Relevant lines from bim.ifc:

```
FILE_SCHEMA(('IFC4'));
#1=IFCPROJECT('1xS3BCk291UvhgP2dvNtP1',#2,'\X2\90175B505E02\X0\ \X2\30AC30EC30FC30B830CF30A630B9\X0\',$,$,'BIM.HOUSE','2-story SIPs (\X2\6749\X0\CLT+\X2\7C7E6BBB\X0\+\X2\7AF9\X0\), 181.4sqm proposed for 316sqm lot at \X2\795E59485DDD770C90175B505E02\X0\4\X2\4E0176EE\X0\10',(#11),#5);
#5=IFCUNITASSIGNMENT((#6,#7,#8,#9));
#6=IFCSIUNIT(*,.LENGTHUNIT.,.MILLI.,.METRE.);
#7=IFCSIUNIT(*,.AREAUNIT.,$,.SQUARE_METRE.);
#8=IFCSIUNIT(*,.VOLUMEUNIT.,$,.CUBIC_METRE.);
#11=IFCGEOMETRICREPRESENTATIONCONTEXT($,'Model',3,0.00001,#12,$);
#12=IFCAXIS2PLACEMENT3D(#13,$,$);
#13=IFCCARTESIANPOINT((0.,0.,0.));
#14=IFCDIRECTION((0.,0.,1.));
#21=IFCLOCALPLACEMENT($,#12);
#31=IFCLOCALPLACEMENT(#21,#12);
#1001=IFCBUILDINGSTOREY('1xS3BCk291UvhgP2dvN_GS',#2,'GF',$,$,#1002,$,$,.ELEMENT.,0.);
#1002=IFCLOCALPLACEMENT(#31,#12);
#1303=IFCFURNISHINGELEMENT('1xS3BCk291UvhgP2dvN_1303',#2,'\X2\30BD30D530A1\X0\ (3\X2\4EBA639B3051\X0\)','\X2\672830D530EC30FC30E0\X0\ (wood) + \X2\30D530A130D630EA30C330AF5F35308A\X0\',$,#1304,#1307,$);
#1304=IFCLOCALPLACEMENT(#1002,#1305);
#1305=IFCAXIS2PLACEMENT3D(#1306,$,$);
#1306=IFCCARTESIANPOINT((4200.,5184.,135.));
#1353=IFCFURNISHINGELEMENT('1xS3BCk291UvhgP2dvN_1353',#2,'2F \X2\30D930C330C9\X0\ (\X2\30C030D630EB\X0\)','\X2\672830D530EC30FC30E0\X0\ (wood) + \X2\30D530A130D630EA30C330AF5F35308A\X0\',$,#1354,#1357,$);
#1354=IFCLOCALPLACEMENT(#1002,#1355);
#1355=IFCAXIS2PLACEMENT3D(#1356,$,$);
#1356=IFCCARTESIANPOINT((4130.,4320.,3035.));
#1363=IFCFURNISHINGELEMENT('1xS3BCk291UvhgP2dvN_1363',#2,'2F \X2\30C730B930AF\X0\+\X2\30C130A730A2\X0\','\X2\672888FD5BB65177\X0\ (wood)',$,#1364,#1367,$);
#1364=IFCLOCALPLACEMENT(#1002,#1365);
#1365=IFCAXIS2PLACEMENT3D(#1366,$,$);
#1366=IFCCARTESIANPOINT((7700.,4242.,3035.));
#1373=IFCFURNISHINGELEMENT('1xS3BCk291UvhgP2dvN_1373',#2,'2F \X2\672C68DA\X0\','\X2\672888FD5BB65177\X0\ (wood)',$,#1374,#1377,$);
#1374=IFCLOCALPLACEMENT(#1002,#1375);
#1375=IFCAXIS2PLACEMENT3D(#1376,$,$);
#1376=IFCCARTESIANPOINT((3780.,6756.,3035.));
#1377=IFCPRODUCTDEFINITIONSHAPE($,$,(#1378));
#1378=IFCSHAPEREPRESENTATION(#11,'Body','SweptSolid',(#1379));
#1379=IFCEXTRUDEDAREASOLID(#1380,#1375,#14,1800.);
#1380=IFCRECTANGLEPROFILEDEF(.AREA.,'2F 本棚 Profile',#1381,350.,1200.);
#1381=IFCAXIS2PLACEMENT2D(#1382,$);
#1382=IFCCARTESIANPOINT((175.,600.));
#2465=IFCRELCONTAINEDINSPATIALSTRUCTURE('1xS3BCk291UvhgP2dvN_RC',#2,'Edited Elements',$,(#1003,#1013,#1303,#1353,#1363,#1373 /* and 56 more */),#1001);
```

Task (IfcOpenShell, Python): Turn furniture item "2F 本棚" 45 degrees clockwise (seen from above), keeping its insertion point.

```python
import ifcopenshell
import ifcopenshell.api.geometry
import ifcopenshell.util.placement

model = ifcopenshell.open("bim.ifc")

item = model.by_guid("1xS3BCk291UvhgP2dvN_1373")
matrix = ifcopenshell.util.placement.get_local_placement(item.ObjectPlacement)
matrix = matrix @ ifcopenshell.util.placement.rotation(-45, "Z")
ifcopenshell.api.geometry.edit_object_placement(model, product=item, matrix=matrix, is_si=False)

print(ifcopenshell.util.placement.get_local_placement(item.ObjectPlacement).round(3) + 0.0)

model.write("bim_edited.ifc")
```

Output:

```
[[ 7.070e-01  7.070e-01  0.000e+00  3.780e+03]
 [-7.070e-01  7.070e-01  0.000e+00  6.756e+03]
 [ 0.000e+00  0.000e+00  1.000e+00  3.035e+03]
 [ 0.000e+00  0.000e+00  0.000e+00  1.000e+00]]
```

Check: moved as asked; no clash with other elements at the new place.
